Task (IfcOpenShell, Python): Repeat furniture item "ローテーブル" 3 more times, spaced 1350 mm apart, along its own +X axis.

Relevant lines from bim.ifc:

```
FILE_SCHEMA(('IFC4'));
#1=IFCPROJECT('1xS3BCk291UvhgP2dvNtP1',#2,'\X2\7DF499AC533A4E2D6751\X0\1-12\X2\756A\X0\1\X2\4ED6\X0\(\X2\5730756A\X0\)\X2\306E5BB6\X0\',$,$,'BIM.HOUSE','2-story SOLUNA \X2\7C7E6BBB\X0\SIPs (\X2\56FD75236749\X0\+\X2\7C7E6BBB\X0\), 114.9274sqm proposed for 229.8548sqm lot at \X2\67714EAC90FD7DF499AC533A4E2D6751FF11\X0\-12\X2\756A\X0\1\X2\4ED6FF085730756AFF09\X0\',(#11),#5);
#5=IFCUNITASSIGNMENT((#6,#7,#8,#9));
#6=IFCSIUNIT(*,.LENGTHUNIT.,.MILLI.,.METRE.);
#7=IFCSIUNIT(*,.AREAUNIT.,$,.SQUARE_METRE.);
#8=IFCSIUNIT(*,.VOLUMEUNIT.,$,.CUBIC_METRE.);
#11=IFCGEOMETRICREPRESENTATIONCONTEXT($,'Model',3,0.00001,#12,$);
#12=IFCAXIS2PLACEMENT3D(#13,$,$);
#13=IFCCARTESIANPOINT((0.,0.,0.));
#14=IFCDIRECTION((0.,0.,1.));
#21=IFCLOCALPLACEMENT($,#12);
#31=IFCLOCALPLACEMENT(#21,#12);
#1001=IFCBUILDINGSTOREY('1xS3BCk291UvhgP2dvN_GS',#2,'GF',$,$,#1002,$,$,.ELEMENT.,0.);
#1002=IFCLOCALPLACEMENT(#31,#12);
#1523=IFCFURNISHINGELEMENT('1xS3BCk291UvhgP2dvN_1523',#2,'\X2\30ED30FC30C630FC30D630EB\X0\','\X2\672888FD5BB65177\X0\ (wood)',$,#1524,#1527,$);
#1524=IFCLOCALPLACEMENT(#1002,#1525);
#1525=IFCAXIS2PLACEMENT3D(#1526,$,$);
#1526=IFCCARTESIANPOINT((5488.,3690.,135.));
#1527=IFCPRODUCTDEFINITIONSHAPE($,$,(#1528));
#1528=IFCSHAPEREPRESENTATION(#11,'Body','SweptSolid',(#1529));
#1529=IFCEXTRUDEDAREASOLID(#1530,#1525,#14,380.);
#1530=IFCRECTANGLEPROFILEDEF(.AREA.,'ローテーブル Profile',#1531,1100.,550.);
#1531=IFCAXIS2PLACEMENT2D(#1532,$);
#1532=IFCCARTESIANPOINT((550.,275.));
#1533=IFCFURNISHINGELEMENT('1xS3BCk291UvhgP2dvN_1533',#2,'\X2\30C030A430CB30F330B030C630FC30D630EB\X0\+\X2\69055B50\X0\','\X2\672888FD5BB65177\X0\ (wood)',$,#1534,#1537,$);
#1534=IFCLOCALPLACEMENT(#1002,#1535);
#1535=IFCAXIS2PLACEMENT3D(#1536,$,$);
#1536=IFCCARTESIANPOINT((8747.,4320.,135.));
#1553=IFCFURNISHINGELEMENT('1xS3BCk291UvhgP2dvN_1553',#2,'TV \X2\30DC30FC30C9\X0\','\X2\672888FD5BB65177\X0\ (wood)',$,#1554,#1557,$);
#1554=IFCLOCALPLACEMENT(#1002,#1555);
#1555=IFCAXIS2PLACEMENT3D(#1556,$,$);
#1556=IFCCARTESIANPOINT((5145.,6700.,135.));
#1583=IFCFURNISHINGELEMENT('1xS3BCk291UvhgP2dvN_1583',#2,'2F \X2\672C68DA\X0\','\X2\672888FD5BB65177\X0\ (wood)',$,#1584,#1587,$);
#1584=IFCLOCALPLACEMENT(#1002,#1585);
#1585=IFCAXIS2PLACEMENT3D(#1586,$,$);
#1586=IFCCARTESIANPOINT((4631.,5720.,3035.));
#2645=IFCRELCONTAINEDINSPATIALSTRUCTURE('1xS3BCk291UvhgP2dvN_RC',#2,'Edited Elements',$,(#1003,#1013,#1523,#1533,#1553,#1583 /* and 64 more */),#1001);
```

```python
import ifcopenshell
import ifcopenshell.api.geometry
import ifcopenshell.api.root
import ifcopenshell.util.element
import ifcopenshell.util.placement
import ifcopenshell.util.unit

model = ifcopenshell.open("bim.ifc")
unit_scale = ifcopenshell.util.unit.calculate_unit_scale(model)


def reuse_history(source, copy):
    """copy_class also copies each property set's owner history, people and application; keep the originals."""
    for rel in copy.IsDefinedBy:
        if rel.is_a("IfcRelDefinesByProperties") and (history := rel.RelatingPropertyDefinition.OwnerHistory):
            rel.RelatingPropertyDefinition.OwnerHistory = source.OwnerHistory
            ifcopenshell.util.element.remove_deep2(model, history)


source = model.by_id(1523)
base = ifcopenshell.util.placement.get_local_placement(source.ObjectPlacement)
step = base[:3, 0] * 1.35 / unit_scale

for i in range(1, 4):
    copy = ifcopenshell.api.root.copy_class(model, product=source)
    copy.Representation = ifcopenshell.util.element.copy_deep(
        model, source.Representation, exclude=["IfcGeometricRepresentationContext", "IfcRepresentationMap"]
    )
    reuse_history(source, copy)
    matrix = base.copy()
    matrix[:3, 3] += i * step
    print("added at", matrix[:3, 3].round(3) + 0.0)
    ifcopenshell.api.geometry.edit_object_placement(model, product=copy, matrix=matrix, is_si=False)

model.write("bim_rev.ifc")
```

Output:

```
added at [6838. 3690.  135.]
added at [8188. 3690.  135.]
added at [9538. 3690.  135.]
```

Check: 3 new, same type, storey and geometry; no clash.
